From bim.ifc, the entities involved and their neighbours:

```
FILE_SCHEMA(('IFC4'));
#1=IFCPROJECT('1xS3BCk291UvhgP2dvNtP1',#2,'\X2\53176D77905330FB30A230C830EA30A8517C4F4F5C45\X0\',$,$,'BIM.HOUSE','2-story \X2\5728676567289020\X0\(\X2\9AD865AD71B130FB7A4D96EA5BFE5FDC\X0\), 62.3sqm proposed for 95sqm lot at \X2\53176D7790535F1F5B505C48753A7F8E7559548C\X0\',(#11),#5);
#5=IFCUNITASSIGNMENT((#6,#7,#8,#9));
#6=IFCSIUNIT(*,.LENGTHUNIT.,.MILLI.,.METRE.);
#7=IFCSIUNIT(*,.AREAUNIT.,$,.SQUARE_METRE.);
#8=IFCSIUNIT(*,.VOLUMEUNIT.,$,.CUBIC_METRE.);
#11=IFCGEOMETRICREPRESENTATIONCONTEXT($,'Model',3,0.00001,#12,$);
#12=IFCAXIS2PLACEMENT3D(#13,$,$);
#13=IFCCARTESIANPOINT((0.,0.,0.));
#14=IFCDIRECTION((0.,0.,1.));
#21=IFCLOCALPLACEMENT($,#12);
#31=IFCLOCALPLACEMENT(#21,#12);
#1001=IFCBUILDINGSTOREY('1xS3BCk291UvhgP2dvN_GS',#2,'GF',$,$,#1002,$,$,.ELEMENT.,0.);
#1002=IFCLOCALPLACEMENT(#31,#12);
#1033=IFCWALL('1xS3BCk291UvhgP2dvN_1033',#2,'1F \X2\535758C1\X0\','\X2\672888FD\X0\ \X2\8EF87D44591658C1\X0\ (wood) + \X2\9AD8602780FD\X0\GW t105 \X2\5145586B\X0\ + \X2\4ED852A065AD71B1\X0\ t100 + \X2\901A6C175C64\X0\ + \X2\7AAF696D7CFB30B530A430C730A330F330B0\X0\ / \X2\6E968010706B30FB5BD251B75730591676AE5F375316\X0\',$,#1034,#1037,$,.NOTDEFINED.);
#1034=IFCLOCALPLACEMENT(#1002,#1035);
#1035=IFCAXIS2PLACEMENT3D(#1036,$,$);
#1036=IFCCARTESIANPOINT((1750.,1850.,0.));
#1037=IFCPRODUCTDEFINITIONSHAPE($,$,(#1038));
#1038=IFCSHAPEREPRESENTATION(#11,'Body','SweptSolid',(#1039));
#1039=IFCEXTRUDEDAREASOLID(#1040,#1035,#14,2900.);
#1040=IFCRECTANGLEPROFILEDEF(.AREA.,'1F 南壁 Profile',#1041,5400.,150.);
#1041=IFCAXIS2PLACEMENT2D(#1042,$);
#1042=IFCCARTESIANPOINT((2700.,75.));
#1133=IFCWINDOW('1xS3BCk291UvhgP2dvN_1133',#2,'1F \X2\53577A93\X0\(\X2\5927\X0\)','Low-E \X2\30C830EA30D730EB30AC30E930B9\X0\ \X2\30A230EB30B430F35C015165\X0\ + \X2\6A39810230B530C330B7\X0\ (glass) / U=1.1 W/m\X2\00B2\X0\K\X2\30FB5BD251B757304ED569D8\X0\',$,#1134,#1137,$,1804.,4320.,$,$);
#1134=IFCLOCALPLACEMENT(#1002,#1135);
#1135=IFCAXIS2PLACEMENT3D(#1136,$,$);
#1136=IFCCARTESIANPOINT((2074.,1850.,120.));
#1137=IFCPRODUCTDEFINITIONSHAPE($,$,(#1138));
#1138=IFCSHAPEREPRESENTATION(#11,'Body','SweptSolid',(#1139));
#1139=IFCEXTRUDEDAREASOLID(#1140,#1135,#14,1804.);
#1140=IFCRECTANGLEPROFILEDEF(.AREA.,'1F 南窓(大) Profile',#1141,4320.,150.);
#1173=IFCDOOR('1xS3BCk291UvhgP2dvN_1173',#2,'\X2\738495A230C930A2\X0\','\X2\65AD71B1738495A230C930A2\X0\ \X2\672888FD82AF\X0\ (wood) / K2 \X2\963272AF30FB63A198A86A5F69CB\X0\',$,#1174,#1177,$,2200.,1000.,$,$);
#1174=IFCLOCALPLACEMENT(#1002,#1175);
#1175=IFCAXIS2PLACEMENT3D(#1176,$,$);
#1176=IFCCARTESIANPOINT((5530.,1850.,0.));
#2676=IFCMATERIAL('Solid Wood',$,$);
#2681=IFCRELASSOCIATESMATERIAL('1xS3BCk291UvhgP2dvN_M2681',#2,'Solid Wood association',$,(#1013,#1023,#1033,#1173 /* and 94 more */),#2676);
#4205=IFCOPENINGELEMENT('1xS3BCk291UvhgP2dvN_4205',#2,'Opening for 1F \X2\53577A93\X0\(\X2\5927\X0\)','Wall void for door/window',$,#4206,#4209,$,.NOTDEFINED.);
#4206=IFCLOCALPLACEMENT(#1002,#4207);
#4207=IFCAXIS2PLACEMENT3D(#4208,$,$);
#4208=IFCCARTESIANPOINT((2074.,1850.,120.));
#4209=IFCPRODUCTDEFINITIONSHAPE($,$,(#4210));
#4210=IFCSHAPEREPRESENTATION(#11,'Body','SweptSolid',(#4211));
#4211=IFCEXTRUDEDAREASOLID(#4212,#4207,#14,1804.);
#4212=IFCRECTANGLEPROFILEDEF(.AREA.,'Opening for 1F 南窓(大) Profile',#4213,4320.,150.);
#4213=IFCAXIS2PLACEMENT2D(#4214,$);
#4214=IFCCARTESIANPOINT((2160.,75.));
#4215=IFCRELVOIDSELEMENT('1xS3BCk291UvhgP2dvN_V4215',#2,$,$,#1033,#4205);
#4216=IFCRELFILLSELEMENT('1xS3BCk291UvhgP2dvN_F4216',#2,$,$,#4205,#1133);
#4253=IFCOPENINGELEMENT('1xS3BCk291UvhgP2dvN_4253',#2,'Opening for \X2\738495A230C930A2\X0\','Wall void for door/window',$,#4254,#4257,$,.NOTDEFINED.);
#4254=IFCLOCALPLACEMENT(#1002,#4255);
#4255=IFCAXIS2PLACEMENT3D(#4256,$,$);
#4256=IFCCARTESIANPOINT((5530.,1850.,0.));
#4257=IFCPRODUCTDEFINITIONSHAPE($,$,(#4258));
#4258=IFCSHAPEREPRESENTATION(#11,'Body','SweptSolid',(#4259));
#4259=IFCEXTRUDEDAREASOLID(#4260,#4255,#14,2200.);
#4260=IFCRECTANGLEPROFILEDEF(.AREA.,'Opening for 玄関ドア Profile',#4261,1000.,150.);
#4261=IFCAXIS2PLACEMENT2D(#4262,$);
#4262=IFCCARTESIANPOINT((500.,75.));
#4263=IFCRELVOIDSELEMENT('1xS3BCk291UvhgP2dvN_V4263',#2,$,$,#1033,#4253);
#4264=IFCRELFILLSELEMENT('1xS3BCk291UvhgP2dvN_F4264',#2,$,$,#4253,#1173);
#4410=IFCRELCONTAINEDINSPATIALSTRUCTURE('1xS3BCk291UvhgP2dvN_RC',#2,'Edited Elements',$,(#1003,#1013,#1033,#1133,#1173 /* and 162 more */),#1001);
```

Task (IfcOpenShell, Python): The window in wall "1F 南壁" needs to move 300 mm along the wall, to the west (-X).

```python
import ifcopenshell
import ifcopenshell.api.geometry
import ifcopenshell.util.placement
import ifcopenshell.util.unit

model = ifcopenshell.open("bim.ifc")
unit_scale = ifcopenshell.util.unit.calculate_unit_scale(model)

window = model.by_guid("1xS3BCk291UvhgP2dvN_1133")
opening = window.FillsVoids[0].RelatingOpeningElement
wall = opening.VoidsElements[0].RelatingBuildingElement

wall_matrix = ifcopenshell.util.placement.get_local_placement(wall.ObjectPlacement)
shift = wall_matrix[:3, 0] * -0.3 / unit_scale
before = ifcopenshell.util.placement.get_local_placement(window.ObjectPlacement)[:3, 3].copy()

# The window is not placed relative to its opening, so move both.
for product in (opening, window):
    matrix = ifcopenshell.util.placement.get_local_placement(product.ObjectPlacement)
    matrix[:3, 3] += shift
    ifcopenshell.api.geometry.edit_object_placement(model, product=product, matrix=matrix, is_si=False)

after = ifcopenshell.util.placement.get_local_placement(window.ObjectPlacement)[:3, 3]
print("window moved by", (after - before).round(3) + 0.0)

model.write("bim-out.ifc")
```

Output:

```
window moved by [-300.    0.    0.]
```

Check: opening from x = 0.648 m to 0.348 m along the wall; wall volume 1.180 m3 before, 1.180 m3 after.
